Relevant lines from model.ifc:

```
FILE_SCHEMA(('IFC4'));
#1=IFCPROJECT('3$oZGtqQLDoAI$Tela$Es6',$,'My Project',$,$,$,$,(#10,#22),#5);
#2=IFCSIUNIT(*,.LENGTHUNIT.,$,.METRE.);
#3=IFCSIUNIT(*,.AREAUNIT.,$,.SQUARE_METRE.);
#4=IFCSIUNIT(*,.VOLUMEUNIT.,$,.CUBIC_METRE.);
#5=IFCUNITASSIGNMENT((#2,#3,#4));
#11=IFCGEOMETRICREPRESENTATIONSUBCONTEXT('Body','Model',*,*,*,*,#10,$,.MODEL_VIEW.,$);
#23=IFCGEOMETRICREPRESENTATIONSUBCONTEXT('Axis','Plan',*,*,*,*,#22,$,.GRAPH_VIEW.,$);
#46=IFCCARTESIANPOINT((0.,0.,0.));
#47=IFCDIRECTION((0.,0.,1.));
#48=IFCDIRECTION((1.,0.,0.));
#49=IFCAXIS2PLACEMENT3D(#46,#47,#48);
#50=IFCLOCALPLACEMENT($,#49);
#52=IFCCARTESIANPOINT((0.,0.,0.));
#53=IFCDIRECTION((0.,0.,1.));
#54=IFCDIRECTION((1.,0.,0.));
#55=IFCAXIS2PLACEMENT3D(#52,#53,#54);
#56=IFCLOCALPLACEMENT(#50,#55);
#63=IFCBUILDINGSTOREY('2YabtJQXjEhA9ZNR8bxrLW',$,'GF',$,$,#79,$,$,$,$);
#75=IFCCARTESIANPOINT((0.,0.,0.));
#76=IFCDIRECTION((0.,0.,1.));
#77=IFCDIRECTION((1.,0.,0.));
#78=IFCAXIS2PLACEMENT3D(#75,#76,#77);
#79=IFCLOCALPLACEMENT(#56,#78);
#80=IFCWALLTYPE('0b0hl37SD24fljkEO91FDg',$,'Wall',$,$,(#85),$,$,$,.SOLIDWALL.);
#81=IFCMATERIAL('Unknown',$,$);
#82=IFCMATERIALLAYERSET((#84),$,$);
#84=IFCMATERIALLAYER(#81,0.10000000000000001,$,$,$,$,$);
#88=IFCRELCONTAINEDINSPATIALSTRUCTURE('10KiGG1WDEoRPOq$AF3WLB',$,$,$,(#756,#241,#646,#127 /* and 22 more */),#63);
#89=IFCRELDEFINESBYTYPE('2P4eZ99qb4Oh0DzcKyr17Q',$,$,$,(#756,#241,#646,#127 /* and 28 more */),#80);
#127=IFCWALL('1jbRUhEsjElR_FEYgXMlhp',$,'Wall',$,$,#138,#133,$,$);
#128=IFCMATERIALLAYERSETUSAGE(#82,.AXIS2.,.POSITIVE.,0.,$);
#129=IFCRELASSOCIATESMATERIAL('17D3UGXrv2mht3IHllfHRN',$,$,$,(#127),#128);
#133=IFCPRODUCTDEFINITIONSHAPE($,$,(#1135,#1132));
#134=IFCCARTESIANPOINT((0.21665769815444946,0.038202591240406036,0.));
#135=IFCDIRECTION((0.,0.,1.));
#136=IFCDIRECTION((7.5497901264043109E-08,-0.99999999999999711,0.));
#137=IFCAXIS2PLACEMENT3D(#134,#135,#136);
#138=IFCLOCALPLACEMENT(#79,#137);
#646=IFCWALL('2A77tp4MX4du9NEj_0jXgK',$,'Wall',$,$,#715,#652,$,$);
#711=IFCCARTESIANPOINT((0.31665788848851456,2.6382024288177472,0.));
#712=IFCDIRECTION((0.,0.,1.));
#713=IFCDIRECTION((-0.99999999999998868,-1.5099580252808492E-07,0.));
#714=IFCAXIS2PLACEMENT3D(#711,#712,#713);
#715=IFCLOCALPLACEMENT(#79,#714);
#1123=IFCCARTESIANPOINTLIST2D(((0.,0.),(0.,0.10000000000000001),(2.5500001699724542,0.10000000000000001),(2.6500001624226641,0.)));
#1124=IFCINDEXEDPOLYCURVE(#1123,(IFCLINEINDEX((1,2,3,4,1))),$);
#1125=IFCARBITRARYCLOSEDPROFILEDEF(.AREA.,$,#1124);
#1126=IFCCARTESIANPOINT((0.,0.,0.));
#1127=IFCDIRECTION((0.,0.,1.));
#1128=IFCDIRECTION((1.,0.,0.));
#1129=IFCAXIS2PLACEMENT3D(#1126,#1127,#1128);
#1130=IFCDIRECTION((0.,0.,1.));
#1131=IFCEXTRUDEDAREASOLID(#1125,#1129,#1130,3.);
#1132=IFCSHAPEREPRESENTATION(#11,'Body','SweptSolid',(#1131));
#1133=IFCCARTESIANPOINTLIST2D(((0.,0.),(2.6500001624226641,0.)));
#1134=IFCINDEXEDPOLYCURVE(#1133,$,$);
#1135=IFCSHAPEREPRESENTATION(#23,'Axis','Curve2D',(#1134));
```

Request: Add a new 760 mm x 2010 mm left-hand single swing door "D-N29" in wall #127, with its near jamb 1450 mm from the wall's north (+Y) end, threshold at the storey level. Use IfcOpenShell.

```python
import numpy as np
import ifcopenshell
import ifcopenshell.api.feature
import ifcopenshell.api.geometry
import ifcopenshell.api.root
import ifcopenshell.api.spatial
import ifcopenshell.geom
import ifcopenshell.util.element
import ifcopenshell.util.placement
import ifcopenshell.util.representation
import ifcopenshell.util.shape
import ifcopenshell.util.unit

model = ifcopenshell.open("model.ifc")
unit_scale = ifcopenshell.util.unit.calculate_unit_scale(model)
settings = ifcopenshell.geom.settings()


def volume(element):
    """Net volume in cubic metres, openings subtracted."""
    shape = ifcopenshell.geom.create_shape(settings, element)
    return ifcopenshell.util.shape.get_volume(shape.geometry)


wall = model.by_guid("1jbRUhEsjElR_FEYgXMlhp")
storey = ifcopenshell.util.element.get_container(wall, ifc_class="IfcBuildingStorey")
context = ifcopenshell.util.representation.get_context(model, "Model", "Body", "MODEL_VIEW")
before = volume(wall)

width, height, from_end, sill = 0.76, 2.01, 1.45, 0.0  # metres

# The wall runs along its own X axis, and the end named is its -X end.
wall_shape = ifcopenshell.geom.create_shape(settings, wall)
x, y, z = ifcopenshell.util.shape.get_vertices(wall_shape.geometry).T
start = x.min() + from_end
face, thickness = float(y.min()), float(y.max() - y.min())
wall_matrix = ifcopenshell.util.placement.get_local_placement(wall.ObjectPlacement)
level = ifcopenshell.util.placement.get_local_placement(storey.ObjectPlacement)[2, 3]


def in_wall(x, y):
    """Placement at x, y metres in the wall's axes, at sill height."""
    matrix = wall_matrix.copy()
    matrix[:, 3] = wall_matrix @ np.array([x / unit_scale, y / unit_scale, 0.0, 1.0])
    matrix[2, 3] = level + sill / unit_scale
    return matrix


# Opening: a box that overshoots both wall faces by 50 mm.
opening = ifcopenshell.api.root.create_entity(model, ifc_class="IfcOpeningElement", predefined_type="OPENING")
box = ifcopenshell.api.geometry.add_wall_representation(
    model, context=context, length=width, height=height, thickness=thickness + 0.1
)
ifcopenshell.api.geometry.assign_representation(model, product=opening, representation=box)
ifcopenshell.api.geometry.edit_object_placement(model, product=opening, matrix=in_wall(start, face - 0.05), is_si=False)
ifcopenshell.api.feature.add_feature(model, feature=opening, element=wall)

door = ifcopenshell.api.root.create_entity(model, ifc_class="IfcDoor", name="D-N29", predefined_type="DOOR")
door.OverallWidth, door.OverallHeight = width / unit_scale, height / unit_scale
door.OperationType = "SINGLE_SWING_LEFT"
body = ifcopenshell.api.geometry.add_door_representation(
    model,
    context=context,
    overall_width=door.OverallWidth,
    overall_height=door.OverallHeight,
    operation_type="SINGLE_SWING_LEFT",
    lining_properties={"LiningDepth": thickness / unit_scale, "ThresholdDepth": thickness / unit_scale},
)
ifcopenshell.api.geometry.assign_representation(model, product=door, representation=body)
ifcopenshell.api.spatial.assign_container(model, products=[door], relating_structure=storey)
ifcopenshell.api.feature.add_filling(model, opening=opening, element=door)

# The lining spans the wall, so the door starts at the wall face.
ifcopenshell.api.geometry.edit_object_placement(model, product=door, matrix=in_wall(start, face), is_si=False)

after = volume(wall)

print(f"wall volume {before:.3f} -> {after:.3f} m3")

model.write("model_edited.ifc")
```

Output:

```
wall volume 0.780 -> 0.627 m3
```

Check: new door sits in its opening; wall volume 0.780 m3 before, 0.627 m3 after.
